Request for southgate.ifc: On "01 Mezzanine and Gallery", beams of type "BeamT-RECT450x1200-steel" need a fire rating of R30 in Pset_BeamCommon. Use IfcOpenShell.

First a look at what the model holds.

```python
import ifcopenshell
import ifcopenshell.util.element

model = ifcopenshell.open("southgate.ifc")
print(model.schema)
storey = next(s for s in model.by_type("IfcBuildingStorey") if s.Name == "01 Mezzanine and Gallery")
beams = [e for e in ifcopenshell.util.element.get_decomposition(storey) if e.is_a("IfcBeam")]
seen = {}
for e in beams:
    element_type = ifcopenshell.util.element.get_type(e)
    key = (element_type.Name if element_type != e and element_type else None, ifcopenshell.util.element.get_pset(e, "Pset_BeamCommon", "FireRating"))
    seen[key] = seen.get(key, 0) + 1
for (name, value), count in sorted(seen.items(), key=str):
    print(count, "x", name, "|", value)
```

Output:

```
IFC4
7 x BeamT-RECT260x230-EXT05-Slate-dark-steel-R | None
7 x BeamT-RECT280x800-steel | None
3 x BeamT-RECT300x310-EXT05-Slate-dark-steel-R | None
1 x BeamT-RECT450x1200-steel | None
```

```python
import ifcopenshell
import ifcopenshell.api.pset
import ifcopenshell.util.element

model = ifcopenshell.open("southgate.ifc")

storey = next(s for s in model.by_type("IfcBuildingStorey") if s.Name == "01 Mezzanine and Gallery")
beams = [e for e in ifcopenshell.util.element.get_decomposition(storey) if e.is_a("IfcBeam")]

count = 0
for e in beams:
    element_type = ifcopenshell.util.element.get_type(e)
    if element_type in (None, e) or element_type.Name != "BeamT-RECT450x1200-steel":
        continue
    # add_pset returns the element's existing set when there is one.
    pset = ifcopenshell.api.pset.add_pset(model, product=e, name="Pset_BeamCommon")
    ifcopenshell.api.pset.edit_pset(model, pset=pset, properties={"FireRating": "R30"})
    count += 1

print(count, "beams updated")

model.write("southgate_updated.ifc")
```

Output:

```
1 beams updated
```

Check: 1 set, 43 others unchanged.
